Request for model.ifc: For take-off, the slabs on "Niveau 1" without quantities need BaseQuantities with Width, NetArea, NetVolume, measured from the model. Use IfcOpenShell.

First a look at what the model holds.

```python
import ifcopenshell
import ifcopenshell.util.element
import ifcopenshell.util.unit

model = ifcopenshell.open("model.ifc")
print(model.schema)
for unit_type in ("LENGTHUNIT", "AREAUNIT", "VOLUMEUNIT"):
    print(unit_type, ifcopenshell.util.unit.calculate_unit_scale(model, unit_type))
storey = next(s for s in model.by_type("IfcBuildingStorey") if s.Name == "Niveau 1")
slabs = [e for e in ifcopenshell.util.element.get_decomposition(storey) if e.is_a("IfcSlab")]
for e in sorted(slabs, key=lambda e: e.id()):
    print(e.id(), e.is_a(), e.Name, list(ifcopenshell.util.element.get_psets(e, qtos_only=True)), sep=" | ")
```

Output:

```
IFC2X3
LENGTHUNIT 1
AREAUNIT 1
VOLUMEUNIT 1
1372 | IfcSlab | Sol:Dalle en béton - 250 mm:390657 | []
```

```python
import ifcopenshell
import ifcopenshell.api.pset
import ifcopenshell.geom
import ifcopenshell.util.element
import ifcopenshell.util.shape
import ifcopenshell.util.unit

model = ifcopenshell.open("model.ifc")
unit_scale = ifcopenshell.util.unit.calculate_unit_scale(model)
area_scale = ifcopenshell.util.unit.calculate_unit_scale(model, "AREAUNIT")
volume_scale = ifcopenshell.util.unit.calculate_unit_scale(model, "VOLUMEUNIT")
settings = ifcopenshell.geom.settings()

storey = next(s for s in model.by_type("IfcBuildingStorey") if s.Name == "Niveau 1")
slabs = [e for e in ifcopenshell.util.element.get_decomposition(storey) if e.is_a("IfcSlab")]

for e in sorted(slabs, key=lambda e: e.id()):
    if ifcopenshell.util.element.get_psets(e, qtos_only=True, should_inherit=False):
        continue
    # Geometry comes back in metres, in the element's own axes.
    shape = ifcopenshell.geom.create_shape(settings, e)
    values = {
        "Width": ifcopenshell.util.shape.get_z(shape.geometry) / unit_scale,
        "NetArea": ifcopenshell.util.shape.get_footprint_area(shape.geometry) / area_scale,
        "NetVolume": ifcopenshell.util.shape.get_volume(shape.geometry) / volume_scale,
    }
    qto = ifcopenshell.api.pset.add_qto(model, product=e, name="BaseQuantities")
    ifcopenshell.api.pset.edit_qto(model, qto=qto, properties=values)
    print(e.id(), {k: round(v, 3) for k, v in values.items()})

model.write("model_rev.ifc")
```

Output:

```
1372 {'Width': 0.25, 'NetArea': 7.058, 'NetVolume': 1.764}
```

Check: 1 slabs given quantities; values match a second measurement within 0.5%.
